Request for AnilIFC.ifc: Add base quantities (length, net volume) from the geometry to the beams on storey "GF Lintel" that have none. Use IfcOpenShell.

First a look at what the model holds.

```python
import ifcopenshell
import ifcopenshell.util.element
import ifcopenshell.util.unit

model = ifcopenshell.open("AnilIFC.ifc")
print(model.schema)
for unit_type in ("LENGTHUNIT", "AREAUNIT", "VOLUMEUNIT"):
    print(unit_type, ifcopenshell.util.unit.calculate_unit_scale(model, unit_type))
storey = next(s for s in model.by_type("IfcBuildingStorey") if s.Name == "GF Lintel")
beams = [e for e in ifcopenshell.util.element.get_decomposition(storey) if e.is_a("IfcBeam")]
for e in sorted(beams, key=lambda e: e.id()):
    print(e.id(), e.is_a(), e.Name, list(ifcopenshell.util.element.get_psets(e, qtos_only=True)), sep=" | ")
```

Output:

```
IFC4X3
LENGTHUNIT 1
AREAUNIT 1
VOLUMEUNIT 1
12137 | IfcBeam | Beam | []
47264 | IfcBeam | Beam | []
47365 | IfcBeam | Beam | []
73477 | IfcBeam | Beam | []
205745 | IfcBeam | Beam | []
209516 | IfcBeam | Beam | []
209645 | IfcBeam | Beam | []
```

```python
import ifcopenshell
import ifcopenshell.api.pset
import ifcopenshell.geom
import ifcopenshell.util.element
import ifcopenshell.util.shape
import ifcopenshell.util.unit

model = ifcopenshell.open("AnilIFC.ifc")
unit_scale = ifcopenshell.util.unit.calculate_unit_scale(model)
volume_scale = ifcopenshell.util.unit.calculate_unit_scale(model, "VOLUMEUNIT")
settings = ifcopenshell.geom.settings()

storey = next(s for s in model.by_type("IfcBuildingStorey") if s.Name == "GF Lintel")
beams = [e for e in ifcopenshell.util.element.get_decomposition(storey) if e.is_a("IfcBeam")]

for e in sorted(beams, key=lambda e: e.id()):
    if ifcopenshell.util.element.get_psets(e, qtos_only=True, should_inherit=False):
        continue
    # Geometry comes back in metres, in the element's own axes.
    shape = ifcopenshell.geom.create_shape(settings, e)
    values = {
        "Length": ifcopenshell.util.shape.get_max_xyz(shape.geometry) / unit_scale,
        "NetVolume": ifcopenshell.util.shape.get_volume(shape.geometry) / volume_scale,
    }
    qto = ifcopenshell.api.pset.add_qto(model, product=e, name="Qto_BeamBaseQuantities")
    ifcopenshell.api.pset.edit_qto(model, qto=qto, properties=values)
    print(e.id(), {k: round(v, 3) for k, v in values.items()})

model.write("AnilIFC-out.ifc")
```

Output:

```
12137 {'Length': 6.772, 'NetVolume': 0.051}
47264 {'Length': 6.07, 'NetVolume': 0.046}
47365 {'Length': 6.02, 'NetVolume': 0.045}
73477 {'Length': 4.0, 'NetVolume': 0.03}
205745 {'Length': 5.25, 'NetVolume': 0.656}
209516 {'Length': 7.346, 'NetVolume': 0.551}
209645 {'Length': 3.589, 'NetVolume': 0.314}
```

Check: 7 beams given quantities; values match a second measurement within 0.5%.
